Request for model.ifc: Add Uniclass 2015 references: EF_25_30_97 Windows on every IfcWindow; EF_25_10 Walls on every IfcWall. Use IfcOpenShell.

First a look at what the model holds.

```python
import ifcopenshell

model = ifcopenshell.open("model.ifc")
print(model.schema)
print("classifications:", [c.Name for c in model.by_type("IfcClassification")])
for ifc_class in ("IfcDoor", "IfcRoof", "IfcStair", "IfcWall", "IfcWindow"):
    print(ifc_class, len(model.by_type(ifc_class)))
```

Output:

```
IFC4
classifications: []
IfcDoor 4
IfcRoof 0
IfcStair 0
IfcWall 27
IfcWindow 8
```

```python
import ifcopenshell
import ifcopenshell.api.classification

model = ifcopenshell.open("model.ifc")

system = ifcopenshell.api.classification.add_classification(model, classification="Uniclass 2015")

codes = {
    "IfcWindow": ("EF_25_30_97", "Windows"),
    "IfcWall": ("EF_25_10", "Walls"),
}
for ifc_class, (code, name) in codes.items():
    products = model.by_type(ifc_class)
    ifcopenshell.api.classification.add_reference(
        model, products=products, classification=system, identification=code, name=name
    )
    print(code, len(products))

model.write("model_edited.ifc")
```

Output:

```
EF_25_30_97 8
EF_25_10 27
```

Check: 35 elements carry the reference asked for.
